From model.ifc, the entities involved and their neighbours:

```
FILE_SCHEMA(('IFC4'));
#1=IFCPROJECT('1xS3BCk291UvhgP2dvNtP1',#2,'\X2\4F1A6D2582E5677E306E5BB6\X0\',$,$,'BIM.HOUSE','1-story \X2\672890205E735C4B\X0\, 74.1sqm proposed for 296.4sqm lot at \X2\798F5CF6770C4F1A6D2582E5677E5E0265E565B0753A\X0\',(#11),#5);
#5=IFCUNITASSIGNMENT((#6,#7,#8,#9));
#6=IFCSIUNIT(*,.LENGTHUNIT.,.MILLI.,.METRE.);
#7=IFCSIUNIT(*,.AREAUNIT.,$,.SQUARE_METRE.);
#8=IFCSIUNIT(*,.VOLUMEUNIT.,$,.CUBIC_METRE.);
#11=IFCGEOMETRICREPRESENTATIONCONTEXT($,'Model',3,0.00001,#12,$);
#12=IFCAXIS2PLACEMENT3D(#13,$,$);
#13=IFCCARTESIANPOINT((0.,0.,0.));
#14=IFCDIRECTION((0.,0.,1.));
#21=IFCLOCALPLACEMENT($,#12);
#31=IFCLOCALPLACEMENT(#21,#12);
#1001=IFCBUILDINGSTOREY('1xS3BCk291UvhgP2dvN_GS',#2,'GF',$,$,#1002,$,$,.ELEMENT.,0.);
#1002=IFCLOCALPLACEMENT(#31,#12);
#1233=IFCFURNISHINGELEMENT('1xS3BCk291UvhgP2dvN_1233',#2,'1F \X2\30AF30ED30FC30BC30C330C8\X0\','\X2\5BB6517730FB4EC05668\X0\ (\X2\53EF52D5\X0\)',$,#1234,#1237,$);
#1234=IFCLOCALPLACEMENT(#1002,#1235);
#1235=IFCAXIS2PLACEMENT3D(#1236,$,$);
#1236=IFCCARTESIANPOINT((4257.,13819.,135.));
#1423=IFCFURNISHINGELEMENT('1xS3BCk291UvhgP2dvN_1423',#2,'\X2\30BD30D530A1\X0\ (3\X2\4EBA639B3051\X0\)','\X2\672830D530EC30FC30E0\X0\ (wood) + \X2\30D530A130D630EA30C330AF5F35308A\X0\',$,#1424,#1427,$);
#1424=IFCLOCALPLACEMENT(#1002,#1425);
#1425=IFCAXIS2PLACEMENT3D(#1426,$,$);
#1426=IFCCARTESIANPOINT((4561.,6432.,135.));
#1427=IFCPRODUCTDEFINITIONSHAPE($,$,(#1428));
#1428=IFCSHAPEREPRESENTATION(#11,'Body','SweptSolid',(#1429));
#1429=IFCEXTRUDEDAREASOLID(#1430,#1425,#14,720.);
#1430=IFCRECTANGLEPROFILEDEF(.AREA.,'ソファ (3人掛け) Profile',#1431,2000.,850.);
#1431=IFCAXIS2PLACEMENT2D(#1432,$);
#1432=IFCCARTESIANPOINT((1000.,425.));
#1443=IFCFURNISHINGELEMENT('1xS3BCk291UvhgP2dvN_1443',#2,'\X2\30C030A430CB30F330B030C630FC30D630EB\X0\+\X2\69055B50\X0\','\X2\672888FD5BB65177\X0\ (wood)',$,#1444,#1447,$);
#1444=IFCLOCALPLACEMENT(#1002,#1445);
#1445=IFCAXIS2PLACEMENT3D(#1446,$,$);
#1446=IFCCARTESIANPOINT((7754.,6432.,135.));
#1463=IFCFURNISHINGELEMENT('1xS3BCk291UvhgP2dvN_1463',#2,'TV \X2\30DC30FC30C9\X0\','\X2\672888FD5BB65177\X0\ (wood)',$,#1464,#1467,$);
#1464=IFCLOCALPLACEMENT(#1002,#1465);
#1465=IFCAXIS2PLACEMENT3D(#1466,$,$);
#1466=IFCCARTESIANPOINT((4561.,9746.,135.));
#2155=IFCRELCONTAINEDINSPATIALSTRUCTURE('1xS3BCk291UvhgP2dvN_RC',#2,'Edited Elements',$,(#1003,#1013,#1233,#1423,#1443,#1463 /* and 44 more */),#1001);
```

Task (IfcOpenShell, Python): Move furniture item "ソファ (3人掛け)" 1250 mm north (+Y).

```python
import ifcopenshell
import ifcopenshell.api.geometry
import ifcopenshell.util.placement

model = ifcopenshell.open("model.ifc")

item = model.by_id(1423)
matrix = ifcopenshell.util.placement.get_local_placement(item.ObjectPlacement)
matrix[1, 3] += 1250.0
ifcopenshell.api.geometry.edit_object_placement(model, product=item, matrix=matrix, is_si=False)

print(ifcopenshell.util.placement.get_local_placement(item.ObjectPlacement).round(3) + 0.0)

model.write("model-out.ifc")
```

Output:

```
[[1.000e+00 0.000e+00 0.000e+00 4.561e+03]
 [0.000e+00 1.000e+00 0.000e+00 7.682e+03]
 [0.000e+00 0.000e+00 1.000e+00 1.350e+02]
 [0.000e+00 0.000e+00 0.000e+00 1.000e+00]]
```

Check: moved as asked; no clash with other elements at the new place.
